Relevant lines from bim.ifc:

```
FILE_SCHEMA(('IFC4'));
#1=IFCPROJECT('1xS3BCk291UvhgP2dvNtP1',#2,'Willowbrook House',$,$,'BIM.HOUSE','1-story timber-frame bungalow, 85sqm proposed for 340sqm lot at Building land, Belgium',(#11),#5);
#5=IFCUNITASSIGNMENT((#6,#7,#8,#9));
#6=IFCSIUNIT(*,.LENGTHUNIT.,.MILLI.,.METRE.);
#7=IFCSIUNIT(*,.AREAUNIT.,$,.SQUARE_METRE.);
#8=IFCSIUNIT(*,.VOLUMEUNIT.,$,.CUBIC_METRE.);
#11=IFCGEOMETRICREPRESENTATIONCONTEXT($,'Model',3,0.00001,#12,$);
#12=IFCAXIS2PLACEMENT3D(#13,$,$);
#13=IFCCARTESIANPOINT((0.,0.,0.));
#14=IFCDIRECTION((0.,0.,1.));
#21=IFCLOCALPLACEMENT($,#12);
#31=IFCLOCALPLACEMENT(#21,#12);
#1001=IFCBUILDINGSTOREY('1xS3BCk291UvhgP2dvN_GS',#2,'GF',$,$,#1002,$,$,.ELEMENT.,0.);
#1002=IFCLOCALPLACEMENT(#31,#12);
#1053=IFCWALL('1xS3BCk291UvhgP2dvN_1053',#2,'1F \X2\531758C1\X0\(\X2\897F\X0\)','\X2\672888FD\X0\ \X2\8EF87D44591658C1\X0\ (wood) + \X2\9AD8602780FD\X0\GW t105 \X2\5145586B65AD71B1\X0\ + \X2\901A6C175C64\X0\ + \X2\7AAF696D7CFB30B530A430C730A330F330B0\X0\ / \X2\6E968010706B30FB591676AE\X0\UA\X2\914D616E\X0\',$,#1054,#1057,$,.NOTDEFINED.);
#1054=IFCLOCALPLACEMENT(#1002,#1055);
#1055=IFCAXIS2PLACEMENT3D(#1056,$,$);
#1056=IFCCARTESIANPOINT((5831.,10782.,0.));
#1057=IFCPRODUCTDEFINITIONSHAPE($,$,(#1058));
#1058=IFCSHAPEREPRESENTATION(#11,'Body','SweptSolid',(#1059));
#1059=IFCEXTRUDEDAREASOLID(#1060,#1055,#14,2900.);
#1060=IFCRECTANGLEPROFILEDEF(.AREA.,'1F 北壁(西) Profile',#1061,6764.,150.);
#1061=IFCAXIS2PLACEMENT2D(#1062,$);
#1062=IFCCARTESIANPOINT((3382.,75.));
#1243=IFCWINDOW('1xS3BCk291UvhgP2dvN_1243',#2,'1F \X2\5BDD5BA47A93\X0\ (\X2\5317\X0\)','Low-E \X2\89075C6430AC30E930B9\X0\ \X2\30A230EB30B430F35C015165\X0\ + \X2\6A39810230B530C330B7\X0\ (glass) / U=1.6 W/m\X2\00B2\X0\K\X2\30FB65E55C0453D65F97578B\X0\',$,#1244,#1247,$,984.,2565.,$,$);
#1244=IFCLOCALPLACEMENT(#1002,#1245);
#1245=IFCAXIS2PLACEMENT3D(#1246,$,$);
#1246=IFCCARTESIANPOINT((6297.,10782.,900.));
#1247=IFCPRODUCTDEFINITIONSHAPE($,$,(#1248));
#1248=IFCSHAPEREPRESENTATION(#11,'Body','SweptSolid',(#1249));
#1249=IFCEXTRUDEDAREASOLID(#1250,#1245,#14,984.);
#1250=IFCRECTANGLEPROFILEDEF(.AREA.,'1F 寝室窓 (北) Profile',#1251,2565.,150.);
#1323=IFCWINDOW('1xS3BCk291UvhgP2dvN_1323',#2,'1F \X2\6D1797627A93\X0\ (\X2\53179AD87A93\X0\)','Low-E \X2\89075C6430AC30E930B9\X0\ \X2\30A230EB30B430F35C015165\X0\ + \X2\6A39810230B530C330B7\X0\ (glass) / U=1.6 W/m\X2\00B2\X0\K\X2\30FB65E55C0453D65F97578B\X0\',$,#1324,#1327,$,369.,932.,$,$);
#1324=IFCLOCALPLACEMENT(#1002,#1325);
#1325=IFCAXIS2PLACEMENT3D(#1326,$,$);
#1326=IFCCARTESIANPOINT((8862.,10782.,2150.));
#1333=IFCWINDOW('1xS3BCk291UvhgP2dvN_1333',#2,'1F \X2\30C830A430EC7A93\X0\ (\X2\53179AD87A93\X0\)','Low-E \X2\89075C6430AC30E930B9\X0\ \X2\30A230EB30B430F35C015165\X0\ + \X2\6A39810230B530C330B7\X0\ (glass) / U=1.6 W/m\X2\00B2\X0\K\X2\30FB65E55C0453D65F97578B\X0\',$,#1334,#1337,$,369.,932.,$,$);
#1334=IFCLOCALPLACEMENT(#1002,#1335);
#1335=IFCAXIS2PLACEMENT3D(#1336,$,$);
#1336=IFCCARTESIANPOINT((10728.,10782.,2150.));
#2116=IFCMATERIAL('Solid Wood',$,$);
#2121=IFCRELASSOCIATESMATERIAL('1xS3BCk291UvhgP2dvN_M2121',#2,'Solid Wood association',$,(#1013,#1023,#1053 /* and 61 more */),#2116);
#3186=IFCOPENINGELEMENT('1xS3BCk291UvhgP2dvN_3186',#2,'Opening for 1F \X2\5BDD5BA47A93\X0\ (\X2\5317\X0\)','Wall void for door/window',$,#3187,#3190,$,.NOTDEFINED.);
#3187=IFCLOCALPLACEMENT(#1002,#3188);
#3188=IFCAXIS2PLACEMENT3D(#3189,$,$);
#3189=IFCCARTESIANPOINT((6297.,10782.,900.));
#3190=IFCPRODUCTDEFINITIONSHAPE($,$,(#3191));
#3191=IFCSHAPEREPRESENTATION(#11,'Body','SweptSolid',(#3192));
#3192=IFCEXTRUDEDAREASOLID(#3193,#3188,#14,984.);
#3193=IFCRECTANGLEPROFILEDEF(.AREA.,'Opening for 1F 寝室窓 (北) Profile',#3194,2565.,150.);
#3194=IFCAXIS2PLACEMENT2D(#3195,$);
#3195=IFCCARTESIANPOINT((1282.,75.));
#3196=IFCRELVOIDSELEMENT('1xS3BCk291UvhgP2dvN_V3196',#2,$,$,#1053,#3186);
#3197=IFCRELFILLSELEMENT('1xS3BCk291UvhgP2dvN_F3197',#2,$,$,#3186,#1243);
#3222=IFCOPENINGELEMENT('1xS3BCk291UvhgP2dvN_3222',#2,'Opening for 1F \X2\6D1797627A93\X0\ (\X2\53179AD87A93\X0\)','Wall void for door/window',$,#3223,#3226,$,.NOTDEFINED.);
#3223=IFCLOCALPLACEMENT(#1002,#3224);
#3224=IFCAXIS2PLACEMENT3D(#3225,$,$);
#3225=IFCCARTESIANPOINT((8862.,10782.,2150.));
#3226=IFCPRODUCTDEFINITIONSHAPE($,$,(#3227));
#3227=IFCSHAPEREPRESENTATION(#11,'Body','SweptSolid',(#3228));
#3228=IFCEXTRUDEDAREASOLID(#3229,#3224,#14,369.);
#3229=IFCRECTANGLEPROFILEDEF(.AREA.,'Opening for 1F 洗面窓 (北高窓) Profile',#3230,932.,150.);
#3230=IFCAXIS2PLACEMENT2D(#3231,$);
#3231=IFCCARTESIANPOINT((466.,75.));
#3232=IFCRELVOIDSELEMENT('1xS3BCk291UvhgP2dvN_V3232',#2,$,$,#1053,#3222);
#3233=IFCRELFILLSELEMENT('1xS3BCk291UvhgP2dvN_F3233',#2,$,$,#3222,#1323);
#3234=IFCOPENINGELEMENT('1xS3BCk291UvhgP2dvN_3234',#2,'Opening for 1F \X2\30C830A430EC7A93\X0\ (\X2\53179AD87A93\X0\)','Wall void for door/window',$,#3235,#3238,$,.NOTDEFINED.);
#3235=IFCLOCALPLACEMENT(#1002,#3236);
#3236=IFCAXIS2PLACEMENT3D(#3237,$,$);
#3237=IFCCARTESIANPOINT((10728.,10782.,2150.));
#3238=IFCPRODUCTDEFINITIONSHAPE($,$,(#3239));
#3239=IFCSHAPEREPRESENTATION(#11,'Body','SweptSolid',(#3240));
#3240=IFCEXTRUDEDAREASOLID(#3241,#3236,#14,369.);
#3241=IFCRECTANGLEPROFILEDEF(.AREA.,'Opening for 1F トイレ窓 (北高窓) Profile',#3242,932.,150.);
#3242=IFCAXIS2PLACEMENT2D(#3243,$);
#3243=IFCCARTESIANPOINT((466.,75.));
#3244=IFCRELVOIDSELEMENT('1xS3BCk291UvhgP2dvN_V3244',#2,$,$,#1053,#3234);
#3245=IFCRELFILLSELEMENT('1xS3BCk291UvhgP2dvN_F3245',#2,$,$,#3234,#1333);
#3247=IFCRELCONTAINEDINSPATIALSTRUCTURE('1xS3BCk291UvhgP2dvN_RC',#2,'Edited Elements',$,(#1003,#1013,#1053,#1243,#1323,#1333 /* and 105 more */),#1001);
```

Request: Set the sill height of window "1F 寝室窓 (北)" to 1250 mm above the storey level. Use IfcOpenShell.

```python
import numpy as np
import ifcopenshell
import ifcopenshell.api.geometry
import ifcopenshell.geom
import ifcopenshell.util.element
import ifcopenshell.util.placement
import ifcopenshell.util.shape
import ifcopenshell.util.unit

model = ifcopenshell.open("bim.ifc")
unit_scale = ifcopenshell.util.unit.calculate_unit_scale(model)

window = model.by_guid("1xS3BCk291UvhgP2dvN_1243")
opening = window.FillsVoids[0].RelatingOpeningElement
storey = ifcopenshell.util.element.get_container(window, ifc_class="IfcBuildingStorey")
level = ifcopenshell.util.placement.get_local_placement(storey.ObjectPlacement)[2, 3]

# The opening's origin need not be at the sill, so measure its lowest point.
shape = ifcopenshell.geom.create_shape(ifcopenshell.geom.settings(), opening)
bottom = ifcopenshell.util.shape.get_shape_bottom_elevation(shape, shape.geometry) / unit_scale
dz = level + 1250.0 - bottom

shift = np.array([0.0, 0.0, dz])
# The window is not placed relative to its opening, so move both.
for product in (opening, window):
    matrix = ifcopenshell.util.placement.get_local_placement(product.ObjectPlacement)
    matrix[:3, 3] += shift
    ifcopenshell.api.geometry.edit_object_placement(model, product=product, matrix=matrix, is_si=False)

print(f"moved by {dz * unit_scale:+.3f} m")

model.write("bim_updated.ifc")
```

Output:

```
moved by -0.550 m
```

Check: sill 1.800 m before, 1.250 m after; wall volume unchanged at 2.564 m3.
